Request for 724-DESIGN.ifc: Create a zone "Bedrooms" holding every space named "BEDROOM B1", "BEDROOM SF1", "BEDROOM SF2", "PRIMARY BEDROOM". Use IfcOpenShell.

First a look at what the model holds.

```python
import ifcopenshell

model = ifcopenshell.open("724-DESIGN.ifc")
print(model.schema)
seen = {}
for space in model.by_type("IfcSpace"):
    seen[space.LongName] = seen.get(space.LongName, 0) + 1
for name, count in sorted(seen.items(), key=str):
    print(count, "x", name)
print("zones:", [z.Name for z in model.by_type("IfcZone")][:20])
```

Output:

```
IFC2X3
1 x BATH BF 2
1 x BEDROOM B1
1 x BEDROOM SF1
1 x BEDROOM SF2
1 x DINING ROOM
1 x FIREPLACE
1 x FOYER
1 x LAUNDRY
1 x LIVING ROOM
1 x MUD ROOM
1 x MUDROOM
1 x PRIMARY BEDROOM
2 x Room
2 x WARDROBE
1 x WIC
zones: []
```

```python
import ifcopenshell
import ifcopenshell.api.group
import ifcopenshell.api.root

model = ifcopenshell.open("724-DESIGN.ifc")

names = {"BEDROOM B1", "BEDROOM SF1", "BEDROOM SF2", "PRIMARY BEDROOM"}
spaces = [s for s in model.by_type("IfcSpace") if s.LongName in names]

zone = ifcopenshell.api.root.create_entity(model, ifc_class="IfcZone", name="Bedrooms")
ifcopenshell.api.group.assign_group(model, products=spaces, group=zone)
print(len(spaces), "spaces in", zone.Name)

model.write("724-DESIGN_v2.ifc")
```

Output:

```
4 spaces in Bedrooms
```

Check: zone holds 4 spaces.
